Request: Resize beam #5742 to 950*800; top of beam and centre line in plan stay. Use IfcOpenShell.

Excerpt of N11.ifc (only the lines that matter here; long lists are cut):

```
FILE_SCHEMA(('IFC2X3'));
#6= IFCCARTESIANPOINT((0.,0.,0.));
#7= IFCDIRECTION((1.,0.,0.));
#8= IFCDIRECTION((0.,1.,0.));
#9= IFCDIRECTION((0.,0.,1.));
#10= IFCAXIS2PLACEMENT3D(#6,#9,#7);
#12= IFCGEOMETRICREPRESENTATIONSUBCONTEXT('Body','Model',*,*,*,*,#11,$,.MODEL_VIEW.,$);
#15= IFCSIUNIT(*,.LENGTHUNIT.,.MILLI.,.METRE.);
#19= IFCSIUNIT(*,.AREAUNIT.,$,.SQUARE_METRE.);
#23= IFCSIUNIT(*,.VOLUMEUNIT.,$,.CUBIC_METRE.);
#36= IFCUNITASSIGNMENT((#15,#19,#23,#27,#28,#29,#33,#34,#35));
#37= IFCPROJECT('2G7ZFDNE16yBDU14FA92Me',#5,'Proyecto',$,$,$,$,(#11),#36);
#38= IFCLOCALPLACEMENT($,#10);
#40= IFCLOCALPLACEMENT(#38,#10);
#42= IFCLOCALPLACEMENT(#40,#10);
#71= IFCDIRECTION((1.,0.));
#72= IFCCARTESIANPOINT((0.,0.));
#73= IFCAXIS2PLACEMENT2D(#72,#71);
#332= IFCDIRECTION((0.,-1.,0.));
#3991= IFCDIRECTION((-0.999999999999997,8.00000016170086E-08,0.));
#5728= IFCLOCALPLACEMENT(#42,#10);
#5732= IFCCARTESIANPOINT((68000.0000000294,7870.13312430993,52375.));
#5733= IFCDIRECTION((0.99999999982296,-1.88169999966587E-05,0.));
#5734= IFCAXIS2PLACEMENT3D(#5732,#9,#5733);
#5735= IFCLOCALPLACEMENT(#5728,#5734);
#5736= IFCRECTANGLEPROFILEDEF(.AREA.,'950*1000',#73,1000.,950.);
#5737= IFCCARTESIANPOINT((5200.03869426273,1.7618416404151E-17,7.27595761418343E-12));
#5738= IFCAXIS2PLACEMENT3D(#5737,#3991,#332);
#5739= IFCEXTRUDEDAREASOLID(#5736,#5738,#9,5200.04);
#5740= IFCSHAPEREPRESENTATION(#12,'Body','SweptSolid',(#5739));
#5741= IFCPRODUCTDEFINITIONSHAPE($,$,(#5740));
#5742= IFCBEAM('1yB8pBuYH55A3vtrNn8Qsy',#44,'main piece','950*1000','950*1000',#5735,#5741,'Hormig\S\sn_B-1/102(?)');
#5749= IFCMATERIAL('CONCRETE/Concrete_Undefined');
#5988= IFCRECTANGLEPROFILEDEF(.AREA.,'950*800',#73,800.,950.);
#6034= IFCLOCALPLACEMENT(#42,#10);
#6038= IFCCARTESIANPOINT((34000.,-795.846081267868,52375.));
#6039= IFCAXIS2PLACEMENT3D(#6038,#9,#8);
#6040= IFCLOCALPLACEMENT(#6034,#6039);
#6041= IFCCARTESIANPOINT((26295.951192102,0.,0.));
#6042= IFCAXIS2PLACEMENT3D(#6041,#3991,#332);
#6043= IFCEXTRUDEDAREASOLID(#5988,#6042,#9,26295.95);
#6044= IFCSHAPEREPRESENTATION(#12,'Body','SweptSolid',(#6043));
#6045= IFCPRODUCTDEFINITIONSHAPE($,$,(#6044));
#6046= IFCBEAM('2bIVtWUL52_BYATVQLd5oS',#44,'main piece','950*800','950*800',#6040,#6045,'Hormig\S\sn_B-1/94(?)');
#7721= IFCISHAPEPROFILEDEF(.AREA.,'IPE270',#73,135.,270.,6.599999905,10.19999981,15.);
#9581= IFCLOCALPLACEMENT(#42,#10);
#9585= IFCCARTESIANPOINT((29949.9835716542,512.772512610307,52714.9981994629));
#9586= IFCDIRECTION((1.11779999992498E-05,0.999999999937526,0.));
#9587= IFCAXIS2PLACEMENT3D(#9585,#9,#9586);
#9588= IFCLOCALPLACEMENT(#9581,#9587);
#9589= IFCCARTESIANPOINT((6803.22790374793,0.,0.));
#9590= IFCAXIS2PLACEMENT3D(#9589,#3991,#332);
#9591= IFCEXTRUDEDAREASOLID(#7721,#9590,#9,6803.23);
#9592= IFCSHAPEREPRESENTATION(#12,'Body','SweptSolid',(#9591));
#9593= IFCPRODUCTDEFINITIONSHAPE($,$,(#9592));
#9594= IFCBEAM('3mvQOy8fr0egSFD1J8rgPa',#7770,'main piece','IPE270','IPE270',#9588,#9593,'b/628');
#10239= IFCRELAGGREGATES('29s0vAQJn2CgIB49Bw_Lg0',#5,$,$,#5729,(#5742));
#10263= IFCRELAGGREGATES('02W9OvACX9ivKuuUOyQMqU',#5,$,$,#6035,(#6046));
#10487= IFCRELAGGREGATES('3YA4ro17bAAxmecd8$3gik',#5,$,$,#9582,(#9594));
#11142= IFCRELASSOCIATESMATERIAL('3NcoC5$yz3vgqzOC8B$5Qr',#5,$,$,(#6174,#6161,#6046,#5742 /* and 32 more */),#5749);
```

```python
import ifcopenshell
import ifcopenshell.util.element
import ifcopenshell.util.representation

model = ifcopenshell.open("N11.ifc")

member = model.by_id(5742)
source = next(p for p in model.by_type("IfcRectangleProfileDef") if p.ProfileName == "950*800")

body = ifcopenshell.util.representation.get_representation(member, "Model", "Body")
solid = body.Items[0]
old_profile = solid.SweptArea

# Copy the section's sizes but keep this member's own profile position.
profile = ifcopenshell.util.element.copy(model, source)
# Profiles are centred, so shift by half the change in depth to hold the top.
shift = (old_profile.YDim - profile.YDim) / 2
x, y = old_profile.Position.Location.Coordinates
up = (0.0, 1.0)  # upwards, in the solid's own plane
location = model.createIfcCartesianPoint((x + up[0] * shift, y + up[1] * shift))
profile.Position = model.createIfcAxis2Placement2D(location, old_profile.Position.RefDirection)
solid.SweptArea = profile
if not model.get_total_inverses(old_profile):
    ifcopenshell.util.element.remove_deep2(model, old_profile)
member.Description = member.Description.replace("950*1000", "950*800")
member.ObjectType = member.ObjectType.replace("950*1000", "950*800")

print(solid.SweptArea)

model.write("N11_edited.ifc")
```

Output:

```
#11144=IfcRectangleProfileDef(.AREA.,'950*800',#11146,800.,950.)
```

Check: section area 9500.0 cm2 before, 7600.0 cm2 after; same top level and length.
